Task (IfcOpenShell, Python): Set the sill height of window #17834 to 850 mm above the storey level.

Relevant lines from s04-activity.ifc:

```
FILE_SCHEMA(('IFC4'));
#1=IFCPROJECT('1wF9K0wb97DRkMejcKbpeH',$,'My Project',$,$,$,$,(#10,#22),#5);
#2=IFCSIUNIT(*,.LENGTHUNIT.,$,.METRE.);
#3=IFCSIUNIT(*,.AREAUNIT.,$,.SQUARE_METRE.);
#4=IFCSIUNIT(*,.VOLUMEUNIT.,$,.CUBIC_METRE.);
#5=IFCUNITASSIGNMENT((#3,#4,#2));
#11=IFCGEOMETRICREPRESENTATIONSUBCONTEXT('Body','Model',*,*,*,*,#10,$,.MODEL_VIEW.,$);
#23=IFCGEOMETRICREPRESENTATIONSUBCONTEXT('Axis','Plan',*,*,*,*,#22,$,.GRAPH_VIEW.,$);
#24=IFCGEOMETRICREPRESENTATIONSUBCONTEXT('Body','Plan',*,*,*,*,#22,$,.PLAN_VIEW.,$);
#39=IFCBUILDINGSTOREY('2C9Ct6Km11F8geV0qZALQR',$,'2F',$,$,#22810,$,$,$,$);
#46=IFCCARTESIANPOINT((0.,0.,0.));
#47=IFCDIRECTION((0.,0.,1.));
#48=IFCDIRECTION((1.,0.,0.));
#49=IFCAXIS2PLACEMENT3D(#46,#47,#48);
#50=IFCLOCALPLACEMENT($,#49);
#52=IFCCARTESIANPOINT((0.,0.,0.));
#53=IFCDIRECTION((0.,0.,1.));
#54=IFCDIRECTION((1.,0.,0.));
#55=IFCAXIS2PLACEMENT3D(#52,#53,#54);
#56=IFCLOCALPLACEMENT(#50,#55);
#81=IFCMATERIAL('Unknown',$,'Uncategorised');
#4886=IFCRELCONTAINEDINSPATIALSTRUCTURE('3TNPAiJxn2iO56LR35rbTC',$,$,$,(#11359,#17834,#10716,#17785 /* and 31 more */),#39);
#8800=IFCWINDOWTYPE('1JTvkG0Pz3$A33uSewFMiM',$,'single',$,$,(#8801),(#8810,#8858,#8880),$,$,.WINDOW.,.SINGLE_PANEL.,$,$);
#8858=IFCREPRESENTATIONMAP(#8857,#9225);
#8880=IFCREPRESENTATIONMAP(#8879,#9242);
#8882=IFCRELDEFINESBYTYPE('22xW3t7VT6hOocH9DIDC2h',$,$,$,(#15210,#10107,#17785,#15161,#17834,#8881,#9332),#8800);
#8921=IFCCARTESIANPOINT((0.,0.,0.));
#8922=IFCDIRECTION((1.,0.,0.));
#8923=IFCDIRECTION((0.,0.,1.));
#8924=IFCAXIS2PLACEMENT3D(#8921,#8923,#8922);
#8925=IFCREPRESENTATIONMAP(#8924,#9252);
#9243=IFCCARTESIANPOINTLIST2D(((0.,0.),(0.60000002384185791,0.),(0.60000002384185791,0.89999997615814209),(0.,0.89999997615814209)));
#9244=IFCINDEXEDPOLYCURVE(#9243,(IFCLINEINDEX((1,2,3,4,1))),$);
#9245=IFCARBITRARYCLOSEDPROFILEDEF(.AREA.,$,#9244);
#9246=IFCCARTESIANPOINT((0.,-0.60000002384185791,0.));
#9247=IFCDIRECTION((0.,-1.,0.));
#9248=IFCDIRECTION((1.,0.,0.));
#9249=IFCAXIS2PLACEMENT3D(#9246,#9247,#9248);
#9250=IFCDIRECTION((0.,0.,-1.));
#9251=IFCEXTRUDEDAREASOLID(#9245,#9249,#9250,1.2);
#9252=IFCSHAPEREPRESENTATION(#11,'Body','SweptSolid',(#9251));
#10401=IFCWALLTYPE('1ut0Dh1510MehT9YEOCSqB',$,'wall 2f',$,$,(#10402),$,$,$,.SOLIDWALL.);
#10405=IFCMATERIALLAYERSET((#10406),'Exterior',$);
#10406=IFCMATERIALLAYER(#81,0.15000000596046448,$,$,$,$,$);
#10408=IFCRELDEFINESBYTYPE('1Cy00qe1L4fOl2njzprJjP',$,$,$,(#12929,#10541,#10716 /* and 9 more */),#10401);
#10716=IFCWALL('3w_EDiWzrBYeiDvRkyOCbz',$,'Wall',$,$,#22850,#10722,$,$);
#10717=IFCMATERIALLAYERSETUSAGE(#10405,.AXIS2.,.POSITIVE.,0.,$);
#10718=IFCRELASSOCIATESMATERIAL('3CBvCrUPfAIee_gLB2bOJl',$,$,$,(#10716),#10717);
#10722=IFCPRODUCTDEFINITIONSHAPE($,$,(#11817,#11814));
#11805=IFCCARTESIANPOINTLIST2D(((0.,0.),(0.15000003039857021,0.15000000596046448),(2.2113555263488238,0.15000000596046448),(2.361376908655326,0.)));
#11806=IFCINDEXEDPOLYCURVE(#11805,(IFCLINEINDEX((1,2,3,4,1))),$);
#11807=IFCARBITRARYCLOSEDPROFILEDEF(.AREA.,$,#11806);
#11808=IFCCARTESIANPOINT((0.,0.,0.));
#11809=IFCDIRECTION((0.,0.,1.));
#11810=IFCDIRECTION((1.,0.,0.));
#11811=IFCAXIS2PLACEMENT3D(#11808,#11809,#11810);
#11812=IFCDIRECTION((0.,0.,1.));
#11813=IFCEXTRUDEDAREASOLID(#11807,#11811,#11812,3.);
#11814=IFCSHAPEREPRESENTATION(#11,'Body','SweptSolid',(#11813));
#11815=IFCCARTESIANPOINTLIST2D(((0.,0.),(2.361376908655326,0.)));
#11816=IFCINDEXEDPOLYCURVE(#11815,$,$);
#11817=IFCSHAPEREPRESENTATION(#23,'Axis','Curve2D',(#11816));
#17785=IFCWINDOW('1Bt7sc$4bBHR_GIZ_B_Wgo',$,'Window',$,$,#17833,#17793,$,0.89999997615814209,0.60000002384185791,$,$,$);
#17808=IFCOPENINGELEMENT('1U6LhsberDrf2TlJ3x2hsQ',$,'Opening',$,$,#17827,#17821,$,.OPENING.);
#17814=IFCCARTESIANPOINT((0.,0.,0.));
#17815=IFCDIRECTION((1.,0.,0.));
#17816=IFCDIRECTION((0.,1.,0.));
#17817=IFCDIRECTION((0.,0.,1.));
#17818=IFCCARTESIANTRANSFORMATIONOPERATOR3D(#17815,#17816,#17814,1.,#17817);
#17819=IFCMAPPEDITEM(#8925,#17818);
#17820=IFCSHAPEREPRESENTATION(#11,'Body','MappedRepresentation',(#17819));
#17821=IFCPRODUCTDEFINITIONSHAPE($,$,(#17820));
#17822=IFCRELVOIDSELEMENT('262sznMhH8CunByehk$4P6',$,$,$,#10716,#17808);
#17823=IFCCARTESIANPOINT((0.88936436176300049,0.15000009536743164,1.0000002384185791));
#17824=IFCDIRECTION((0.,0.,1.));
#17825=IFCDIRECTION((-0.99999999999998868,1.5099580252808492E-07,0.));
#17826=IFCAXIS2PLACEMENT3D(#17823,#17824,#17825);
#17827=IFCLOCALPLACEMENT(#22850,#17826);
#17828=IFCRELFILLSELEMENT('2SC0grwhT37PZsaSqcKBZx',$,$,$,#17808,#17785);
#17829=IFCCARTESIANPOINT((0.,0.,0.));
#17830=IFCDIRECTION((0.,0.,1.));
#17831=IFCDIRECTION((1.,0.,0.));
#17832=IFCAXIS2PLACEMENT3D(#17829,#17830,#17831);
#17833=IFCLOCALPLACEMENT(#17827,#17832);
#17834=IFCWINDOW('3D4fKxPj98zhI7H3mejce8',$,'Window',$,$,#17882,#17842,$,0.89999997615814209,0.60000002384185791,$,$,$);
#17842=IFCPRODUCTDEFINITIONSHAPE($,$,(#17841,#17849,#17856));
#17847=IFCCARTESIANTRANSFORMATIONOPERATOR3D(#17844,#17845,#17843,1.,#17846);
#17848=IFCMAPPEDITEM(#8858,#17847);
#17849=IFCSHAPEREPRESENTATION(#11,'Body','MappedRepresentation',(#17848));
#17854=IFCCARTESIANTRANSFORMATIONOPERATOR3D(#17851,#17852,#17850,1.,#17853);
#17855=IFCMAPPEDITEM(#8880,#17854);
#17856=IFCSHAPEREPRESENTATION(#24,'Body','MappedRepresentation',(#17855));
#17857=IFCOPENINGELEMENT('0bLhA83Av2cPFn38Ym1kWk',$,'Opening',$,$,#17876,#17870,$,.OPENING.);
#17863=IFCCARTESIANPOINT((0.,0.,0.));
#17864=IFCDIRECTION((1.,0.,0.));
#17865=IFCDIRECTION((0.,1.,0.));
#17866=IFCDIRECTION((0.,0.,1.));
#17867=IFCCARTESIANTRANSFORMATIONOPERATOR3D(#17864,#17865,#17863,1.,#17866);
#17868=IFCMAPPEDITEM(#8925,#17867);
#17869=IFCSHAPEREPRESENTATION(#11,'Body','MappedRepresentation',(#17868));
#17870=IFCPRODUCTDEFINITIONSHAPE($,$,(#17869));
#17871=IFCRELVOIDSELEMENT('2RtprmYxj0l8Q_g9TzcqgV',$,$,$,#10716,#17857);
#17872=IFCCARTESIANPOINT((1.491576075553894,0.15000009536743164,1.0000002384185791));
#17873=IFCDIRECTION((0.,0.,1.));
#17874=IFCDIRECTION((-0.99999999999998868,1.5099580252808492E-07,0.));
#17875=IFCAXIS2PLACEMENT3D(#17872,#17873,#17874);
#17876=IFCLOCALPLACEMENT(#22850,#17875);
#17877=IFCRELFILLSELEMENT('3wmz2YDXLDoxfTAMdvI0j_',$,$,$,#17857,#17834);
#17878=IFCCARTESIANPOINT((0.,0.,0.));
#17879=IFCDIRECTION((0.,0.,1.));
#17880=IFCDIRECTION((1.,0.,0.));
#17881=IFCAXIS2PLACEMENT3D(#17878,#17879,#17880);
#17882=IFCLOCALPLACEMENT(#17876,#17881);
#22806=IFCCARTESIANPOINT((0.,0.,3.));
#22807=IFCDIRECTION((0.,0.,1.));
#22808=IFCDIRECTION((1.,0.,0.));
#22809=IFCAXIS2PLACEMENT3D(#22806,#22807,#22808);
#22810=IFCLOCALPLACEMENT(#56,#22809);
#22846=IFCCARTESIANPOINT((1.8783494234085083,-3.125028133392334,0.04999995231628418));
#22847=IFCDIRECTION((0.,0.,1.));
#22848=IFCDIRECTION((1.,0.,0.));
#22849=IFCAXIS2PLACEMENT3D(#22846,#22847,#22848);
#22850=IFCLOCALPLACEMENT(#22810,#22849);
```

```python
import numpy as np
import ifcopenshell
import ifcopenshell.api.geometry
import ifcopenshell.geom
import ifcopenshell.util.element
import ifcopenshell.util.placement
import ifcopenshell.util.shape
import ifcopenshell.util.unit

model = ifcopenshell.open("s04-activity.ifc")
unit_scale = ifcopenshell.util.unit.calculate_unit_scale(model)

window = model.by_guid("3D4fKxPj98zhI7H3mejce8")
opening = window.FillsVoids[0].RelatingOpeningElement
storey = ifcopenshell.util.element.get_container(window, ifc_class="IfcBuildingStorey")
level = ifcopenshell.util.placement.get_local_placement(storey.ObjectPlacement)[2, 3]

# The opening's origin need not be at the sill, so measure its lowest point.
shape = ifcopenshell.geom.create_shape(ifcopenshell.geom.settings(), opening)
bottom = ifcopenshell.util.shape.get_shape_bottom_elevation(shape, shape.geometry) / unit_scale
dz = level + 0.85 - bottom

shift = np.array([0.0, 0.0, dz])
# The window is placed relative to its opening, so it follows when the opening moves.
matrix = ifcopenshell.util.placement.get_local_placement(opening.ObjectPlacement)
matrix[:3, 3] += shift
ifcopenshell.api.geometry.edit_object_placement(
    model, product=opening, matrix=matrix, is_si=False, should_transform_children=True
)

print(f"moved by {dz * unit_scale:+.3f} m")

model.write("s04-activity_edited.ifc")
```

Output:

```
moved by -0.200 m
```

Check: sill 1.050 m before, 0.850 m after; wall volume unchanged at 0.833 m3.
